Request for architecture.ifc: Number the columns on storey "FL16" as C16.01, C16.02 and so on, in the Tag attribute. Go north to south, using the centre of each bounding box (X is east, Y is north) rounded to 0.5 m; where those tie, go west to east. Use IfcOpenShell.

First a look at what the model holds.

```python
import ifcopenshell
import ifcopenshell.util.element
import ifcopenshell.util.placement

model = ifcopenshell.open("architecture.ifc")
print(model.schema)
storey = next(s for s in model.by_type("IfcBuildingStorey") if s.Name == "FL16")
columns = [e for e in ifcopenshell.util.element.get_decomposition(storey) if e.is_a("IfcColumn")]
for e in sorted(columns, key=lambda e: e.id()):
    origin = ifcopenshell.util.placement.get_local_placement(e.ObjectPlacement)[:3, 3]
    print(e.id(), e.Tag, e.Name, origin.round(2) + 0.0, sep=" | ")
```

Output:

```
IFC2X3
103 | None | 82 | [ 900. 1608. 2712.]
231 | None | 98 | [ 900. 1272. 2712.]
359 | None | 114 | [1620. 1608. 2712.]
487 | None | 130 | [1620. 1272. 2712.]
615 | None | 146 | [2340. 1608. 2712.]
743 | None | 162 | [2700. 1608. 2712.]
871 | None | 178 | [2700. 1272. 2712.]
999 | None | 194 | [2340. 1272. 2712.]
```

```python
import ifcopenshell
import ifcopenshell.geom
import ifcopenshell.util.element
import ifcopenshell.util.shape

model = ifcopenshell.open("architecture.ifc")
settings = ifcopenshell.geom.settings()
settings.set("use-world-coords", True)


def centre(element):
    shape = ifcopenshell.geom.create_shape(settings, element)
    return ifcopenshell.util.shape.get_bbox_centroid(shape.geometry)


storey = next(s for s in model.by_type("IfcBuildingStorey") if s.Name == "FL16")
columns = [e for e in ifcopenshell.util.element.get_decomposition(storey) if e.is_a("IfcColumn")]

# Insertion points can sit at a corner or the storey origin, so sort by the geometry (in metres).
centres = {e: centre(e) for e in columns}
columns.sort(key=lambda e: (-round(centres[e][1] / 0.5), centres[e][0]))

for i, e in enumerate(columns, start=1):
    number = f"C16.{i:02d}"
    e.Tag = number
    print(e.id(), number)

model.write("architecture_updated.ifc")
```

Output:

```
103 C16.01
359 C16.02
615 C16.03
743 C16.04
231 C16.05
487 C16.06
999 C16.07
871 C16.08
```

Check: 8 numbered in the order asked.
